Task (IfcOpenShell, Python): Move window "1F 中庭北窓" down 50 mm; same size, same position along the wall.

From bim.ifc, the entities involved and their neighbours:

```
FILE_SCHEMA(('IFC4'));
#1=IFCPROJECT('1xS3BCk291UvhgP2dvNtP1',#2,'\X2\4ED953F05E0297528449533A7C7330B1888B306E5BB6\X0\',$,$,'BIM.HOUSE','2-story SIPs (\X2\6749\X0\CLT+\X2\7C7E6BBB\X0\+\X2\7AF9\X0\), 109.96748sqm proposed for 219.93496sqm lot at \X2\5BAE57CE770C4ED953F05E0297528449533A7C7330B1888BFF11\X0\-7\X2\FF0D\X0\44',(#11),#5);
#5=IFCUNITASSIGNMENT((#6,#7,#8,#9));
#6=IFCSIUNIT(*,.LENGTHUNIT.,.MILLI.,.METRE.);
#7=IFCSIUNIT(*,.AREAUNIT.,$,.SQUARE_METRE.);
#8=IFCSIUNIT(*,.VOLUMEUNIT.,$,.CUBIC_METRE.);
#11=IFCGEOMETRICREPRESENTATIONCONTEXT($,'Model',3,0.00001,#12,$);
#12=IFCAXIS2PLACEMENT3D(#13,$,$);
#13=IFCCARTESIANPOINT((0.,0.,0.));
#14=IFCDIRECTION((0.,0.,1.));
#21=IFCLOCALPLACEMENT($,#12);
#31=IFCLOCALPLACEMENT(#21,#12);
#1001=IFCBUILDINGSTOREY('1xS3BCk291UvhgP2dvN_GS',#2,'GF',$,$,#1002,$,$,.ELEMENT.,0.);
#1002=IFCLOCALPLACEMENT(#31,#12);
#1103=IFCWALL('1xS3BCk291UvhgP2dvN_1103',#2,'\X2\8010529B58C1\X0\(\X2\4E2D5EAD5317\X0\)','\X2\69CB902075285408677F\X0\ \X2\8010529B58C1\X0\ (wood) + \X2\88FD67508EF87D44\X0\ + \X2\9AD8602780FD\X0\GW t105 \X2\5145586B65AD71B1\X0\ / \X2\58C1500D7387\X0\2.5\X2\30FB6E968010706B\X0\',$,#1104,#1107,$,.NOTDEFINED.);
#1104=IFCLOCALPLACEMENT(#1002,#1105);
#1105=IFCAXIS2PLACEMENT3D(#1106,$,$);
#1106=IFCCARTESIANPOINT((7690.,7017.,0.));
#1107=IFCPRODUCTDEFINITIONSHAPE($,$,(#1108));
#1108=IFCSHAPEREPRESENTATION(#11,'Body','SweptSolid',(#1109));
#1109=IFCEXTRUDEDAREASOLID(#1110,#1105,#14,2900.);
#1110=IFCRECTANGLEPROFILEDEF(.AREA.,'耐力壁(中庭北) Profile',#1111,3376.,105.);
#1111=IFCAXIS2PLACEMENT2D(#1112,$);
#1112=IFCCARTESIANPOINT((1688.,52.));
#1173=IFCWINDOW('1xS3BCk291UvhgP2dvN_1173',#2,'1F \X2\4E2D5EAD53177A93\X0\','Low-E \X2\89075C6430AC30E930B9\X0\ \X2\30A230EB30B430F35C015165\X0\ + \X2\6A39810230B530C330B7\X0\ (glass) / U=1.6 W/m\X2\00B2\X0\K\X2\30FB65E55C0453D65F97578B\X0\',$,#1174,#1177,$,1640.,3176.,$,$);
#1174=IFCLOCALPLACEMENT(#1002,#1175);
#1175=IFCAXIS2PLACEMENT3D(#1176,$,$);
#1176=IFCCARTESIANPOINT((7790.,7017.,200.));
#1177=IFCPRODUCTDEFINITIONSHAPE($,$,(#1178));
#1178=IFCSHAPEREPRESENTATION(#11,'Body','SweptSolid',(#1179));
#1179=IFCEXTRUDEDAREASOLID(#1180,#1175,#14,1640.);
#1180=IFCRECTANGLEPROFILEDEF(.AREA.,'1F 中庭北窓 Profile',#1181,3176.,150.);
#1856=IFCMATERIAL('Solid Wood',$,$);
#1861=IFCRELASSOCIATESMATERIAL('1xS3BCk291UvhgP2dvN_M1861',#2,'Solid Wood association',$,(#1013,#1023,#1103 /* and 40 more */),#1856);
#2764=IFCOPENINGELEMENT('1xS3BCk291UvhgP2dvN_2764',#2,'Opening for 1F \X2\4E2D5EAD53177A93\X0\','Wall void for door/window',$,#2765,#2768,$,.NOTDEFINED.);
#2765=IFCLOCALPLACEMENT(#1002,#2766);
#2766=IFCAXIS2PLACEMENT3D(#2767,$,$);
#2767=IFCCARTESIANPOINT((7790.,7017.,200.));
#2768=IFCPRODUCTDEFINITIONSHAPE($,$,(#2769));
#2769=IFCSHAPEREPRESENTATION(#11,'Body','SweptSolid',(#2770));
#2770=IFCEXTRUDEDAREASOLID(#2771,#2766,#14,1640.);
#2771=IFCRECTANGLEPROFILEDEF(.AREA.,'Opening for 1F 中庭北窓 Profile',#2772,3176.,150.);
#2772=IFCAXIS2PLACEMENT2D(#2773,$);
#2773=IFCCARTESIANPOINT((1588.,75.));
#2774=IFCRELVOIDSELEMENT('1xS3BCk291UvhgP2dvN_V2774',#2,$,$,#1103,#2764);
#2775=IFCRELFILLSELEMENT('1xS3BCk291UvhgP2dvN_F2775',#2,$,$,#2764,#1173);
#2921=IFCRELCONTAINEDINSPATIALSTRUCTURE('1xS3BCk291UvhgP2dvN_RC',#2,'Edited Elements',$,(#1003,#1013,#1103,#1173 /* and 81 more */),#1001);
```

```python
import numpy as np
import ifcopenshell
import ifcopenshell.api.geometry
import ifcopenshell.util.placement
import ifcopenshell.util.unit

model = ifcopenshell.open("bim.ifc")
unit_scale = ifcopenshell.util.unit.calculate_unit_scale(model)

window = model.by_id(1173)
opening = window.FillsVoids[0].RelatingOpeningElement
dz = -0.05 / unit_scale

shift = np.array([0.0, 0.0, dz])
# The window is not placed relative to its opening, so move both.
for product in (opening, window):
    matrix = ifcopenshell.util.placement.get_local_placement(product.ObjectPlacement)
    matrix[:3, 3] += shift
    ifcopenshell.api.geometry.edit_object_placement(model, product=product, matrix=matrix, is_si=False)

print(f"moved by {dz * unit_scale:+.3f} m")

model.write("bim-out.ifc")
```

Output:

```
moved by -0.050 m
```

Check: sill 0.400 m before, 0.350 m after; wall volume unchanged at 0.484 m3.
